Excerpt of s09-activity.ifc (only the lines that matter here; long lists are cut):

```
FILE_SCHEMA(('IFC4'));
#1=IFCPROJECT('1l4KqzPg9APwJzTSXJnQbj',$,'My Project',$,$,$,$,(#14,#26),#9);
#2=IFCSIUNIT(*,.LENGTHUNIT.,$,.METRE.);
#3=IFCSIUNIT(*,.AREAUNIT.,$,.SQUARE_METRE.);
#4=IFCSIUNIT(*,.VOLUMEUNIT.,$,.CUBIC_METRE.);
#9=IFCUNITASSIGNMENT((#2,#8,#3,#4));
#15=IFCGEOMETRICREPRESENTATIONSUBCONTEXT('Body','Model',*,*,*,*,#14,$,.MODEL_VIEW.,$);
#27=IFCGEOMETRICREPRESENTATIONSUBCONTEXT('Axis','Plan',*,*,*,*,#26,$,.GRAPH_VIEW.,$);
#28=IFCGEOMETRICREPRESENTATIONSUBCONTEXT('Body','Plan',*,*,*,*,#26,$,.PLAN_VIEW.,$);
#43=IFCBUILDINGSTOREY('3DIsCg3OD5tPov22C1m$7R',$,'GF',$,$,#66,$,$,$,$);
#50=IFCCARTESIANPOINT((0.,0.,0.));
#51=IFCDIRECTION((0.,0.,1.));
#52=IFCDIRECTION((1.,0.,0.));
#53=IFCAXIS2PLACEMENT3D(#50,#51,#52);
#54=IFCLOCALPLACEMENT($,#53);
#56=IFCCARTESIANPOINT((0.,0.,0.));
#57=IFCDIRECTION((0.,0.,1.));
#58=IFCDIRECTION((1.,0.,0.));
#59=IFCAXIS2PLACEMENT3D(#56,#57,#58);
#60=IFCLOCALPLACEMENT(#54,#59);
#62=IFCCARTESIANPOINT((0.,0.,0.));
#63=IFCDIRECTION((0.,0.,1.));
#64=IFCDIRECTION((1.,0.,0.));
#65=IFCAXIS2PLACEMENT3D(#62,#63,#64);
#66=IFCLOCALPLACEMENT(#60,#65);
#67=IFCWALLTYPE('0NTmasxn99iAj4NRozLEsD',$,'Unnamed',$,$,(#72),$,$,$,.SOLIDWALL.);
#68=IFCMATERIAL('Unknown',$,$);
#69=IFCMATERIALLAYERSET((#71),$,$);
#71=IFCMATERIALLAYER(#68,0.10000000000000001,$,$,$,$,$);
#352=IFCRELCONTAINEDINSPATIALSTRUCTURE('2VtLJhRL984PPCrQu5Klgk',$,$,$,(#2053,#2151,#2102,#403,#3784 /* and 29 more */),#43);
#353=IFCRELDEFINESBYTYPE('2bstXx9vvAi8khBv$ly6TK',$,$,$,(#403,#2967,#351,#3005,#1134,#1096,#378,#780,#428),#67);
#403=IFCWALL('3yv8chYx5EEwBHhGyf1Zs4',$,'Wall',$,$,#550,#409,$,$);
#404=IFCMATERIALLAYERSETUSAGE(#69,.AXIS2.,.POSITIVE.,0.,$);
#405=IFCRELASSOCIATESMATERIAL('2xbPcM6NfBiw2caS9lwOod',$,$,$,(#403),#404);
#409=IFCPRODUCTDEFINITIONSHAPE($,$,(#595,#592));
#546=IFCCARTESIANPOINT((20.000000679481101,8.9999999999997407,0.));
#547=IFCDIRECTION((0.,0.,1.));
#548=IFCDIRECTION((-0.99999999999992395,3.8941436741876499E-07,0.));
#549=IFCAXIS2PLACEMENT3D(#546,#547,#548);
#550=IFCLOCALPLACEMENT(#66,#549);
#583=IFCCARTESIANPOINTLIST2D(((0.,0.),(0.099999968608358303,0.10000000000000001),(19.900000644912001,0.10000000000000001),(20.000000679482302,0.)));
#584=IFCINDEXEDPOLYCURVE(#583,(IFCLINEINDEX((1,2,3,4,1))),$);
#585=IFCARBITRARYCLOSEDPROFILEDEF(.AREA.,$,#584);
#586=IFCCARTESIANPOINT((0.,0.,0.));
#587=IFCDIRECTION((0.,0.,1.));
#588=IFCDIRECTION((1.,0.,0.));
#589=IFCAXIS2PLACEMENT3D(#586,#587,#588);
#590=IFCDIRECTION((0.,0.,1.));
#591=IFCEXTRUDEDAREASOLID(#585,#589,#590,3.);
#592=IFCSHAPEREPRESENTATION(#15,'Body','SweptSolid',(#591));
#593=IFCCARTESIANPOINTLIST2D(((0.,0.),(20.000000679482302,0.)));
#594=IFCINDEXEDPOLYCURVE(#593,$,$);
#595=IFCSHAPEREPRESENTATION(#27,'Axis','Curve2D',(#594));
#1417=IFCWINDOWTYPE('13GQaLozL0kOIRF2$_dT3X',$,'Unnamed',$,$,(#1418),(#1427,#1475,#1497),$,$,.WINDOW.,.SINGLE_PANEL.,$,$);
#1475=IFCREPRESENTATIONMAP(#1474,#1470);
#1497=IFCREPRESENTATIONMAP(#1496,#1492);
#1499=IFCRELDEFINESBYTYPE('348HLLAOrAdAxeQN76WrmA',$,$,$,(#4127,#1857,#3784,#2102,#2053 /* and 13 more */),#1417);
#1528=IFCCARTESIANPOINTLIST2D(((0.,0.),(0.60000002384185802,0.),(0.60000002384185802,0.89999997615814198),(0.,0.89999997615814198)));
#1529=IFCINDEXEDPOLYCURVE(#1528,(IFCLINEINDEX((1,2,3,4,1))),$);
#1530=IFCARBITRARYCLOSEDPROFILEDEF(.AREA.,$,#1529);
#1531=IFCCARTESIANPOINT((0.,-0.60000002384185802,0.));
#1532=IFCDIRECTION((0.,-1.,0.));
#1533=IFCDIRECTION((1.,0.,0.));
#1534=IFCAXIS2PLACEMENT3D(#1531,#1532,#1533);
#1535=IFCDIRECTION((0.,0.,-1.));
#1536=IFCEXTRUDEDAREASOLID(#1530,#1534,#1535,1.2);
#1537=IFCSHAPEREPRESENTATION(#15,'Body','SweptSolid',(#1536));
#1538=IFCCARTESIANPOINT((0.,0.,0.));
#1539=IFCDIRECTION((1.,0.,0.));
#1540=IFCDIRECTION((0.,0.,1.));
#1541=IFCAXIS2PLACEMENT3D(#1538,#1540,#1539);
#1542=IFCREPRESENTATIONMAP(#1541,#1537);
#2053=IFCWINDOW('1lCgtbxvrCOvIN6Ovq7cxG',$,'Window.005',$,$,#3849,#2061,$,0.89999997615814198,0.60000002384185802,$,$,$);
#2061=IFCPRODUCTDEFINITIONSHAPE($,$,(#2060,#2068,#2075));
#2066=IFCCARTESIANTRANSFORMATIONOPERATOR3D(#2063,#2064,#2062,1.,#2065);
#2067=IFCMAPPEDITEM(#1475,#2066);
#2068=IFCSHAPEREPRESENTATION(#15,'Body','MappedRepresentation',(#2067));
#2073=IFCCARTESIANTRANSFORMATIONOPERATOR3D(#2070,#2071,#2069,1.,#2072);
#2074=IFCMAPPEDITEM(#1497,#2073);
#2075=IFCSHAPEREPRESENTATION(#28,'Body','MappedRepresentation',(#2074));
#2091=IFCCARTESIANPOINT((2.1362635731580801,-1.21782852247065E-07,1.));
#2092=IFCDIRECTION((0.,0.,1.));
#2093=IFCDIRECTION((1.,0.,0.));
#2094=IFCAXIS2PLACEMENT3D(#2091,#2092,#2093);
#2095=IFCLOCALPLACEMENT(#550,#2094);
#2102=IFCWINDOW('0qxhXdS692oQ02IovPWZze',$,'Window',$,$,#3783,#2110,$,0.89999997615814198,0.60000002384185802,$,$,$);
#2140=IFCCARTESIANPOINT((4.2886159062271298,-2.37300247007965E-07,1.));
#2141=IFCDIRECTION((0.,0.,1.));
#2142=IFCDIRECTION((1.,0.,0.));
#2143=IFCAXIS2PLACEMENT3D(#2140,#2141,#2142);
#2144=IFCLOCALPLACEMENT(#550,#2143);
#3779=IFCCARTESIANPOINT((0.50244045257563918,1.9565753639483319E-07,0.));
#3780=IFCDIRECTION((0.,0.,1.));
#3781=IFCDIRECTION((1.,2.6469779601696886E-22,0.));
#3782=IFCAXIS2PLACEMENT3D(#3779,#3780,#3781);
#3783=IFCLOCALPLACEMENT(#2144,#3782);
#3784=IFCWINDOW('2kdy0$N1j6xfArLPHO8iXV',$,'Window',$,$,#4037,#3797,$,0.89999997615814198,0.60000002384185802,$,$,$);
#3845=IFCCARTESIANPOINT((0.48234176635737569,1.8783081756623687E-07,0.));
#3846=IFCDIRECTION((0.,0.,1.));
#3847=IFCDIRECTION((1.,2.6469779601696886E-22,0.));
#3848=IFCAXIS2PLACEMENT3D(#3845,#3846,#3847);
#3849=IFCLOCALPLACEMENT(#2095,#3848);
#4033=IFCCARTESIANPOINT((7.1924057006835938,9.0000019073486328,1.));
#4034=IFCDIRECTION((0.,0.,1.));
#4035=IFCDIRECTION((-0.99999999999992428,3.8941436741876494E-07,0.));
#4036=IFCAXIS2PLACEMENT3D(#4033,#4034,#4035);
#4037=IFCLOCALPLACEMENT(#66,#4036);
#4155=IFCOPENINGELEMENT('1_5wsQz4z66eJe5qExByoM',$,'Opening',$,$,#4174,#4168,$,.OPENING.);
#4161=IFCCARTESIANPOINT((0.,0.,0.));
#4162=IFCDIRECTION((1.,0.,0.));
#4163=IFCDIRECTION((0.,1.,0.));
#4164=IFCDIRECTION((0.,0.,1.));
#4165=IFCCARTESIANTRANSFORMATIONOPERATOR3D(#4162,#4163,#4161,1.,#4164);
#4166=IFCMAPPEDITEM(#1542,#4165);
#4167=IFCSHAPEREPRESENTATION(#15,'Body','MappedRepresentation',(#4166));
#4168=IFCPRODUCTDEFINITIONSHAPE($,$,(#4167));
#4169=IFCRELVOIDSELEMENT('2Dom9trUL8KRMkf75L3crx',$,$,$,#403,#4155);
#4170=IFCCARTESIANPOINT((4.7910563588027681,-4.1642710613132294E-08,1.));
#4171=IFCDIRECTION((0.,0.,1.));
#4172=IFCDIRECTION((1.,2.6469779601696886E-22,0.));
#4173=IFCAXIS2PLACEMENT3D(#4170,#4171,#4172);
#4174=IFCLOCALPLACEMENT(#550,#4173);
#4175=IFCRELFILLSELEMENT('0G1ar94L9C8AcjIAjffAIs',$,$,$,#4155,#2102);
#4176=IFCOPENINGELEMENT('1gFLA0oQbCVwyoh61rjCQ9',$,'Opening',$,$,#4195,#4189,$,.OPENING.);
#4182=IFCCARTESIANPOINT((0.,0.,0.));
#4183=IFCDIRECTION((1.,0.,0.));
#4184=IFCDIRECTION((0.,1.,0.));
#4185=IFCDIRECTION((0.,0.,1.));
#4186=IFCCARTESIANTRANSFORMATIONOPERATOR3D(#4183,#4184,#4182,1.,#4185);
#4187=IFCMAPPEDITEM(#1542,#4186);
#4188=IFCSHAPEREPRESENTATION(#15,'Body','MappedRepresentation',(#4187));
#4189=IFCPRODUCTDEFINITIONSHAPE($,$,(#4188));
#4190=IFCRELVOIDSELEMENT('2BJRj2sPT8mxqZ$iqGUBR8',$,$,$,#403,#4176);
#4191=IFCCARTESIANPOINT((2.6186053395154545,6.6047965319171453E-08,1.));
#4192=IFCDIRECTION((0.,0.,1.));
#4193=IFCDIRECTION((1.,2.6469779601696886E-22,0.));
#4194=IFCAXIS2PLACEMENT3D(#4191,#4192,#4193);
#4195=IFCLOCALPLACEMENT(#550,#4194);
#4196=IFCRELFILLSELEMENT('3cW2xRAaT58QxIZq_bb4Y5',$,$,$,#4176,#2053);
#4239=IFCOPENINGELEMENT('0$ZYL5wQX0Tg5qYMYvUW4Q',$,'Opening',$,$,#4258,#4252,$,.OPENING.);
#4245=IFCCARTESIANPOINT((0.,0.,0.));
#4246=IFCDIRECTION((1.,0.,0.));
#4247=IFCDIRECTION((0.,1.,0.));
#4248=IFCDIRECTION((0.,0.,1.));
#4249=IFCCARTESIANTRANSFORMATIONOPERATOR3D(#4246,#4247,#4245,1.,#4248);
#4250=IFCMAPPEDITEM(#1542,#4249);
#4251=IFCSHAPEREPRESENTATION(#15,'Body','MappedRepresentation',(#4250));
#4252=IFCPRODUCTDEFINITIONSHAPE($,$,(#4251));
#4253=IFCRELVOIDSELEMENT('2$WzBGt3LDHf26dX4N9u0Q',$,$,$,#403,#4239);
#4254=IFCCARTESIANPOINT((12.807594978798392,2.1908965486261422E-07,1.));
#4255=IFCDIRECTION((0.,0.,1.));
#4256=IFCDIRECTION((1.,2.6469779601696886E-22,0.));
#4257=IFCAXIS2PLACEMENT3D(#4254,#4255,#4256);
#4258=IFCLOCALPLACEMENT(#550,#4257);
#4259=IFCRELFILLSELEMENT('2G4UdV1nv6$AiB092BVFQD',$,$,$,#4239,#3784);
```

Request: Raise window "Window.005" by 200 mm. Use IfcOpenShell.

```python
import numpy as np
import ifcopenshell
import ifcopenshell.api.geometry
import ifcopenshell.util.placement
import ifcopenshell.util.unit

model = ifcopenshell.open("s09-activity.ifc")
unit_scale = ifcopenshell.util.unit.calculate_unit_scale(model)

window = model.by_id(2053)
opening = window.FillsVoids[0].RelatingOpeningElement
dz = 0.2 / unit_scale

shift = np.array([0.0, 0.0, dz])
# The window is not placed relative to its opening, so move both.
for product in (opening, window):
    matrix = ifcopenshell.util.placement.get_local_placement(product.ObjectPlacement)
    matrix[:3, 3] += shift
    ifcopenshell.api.geometry.edit_object_placement(model, product=product, matrix=matrix, is_si=False)

print(f"moved by {dz * unit_scale:+.3f} m")

model.write("s09-activity_updated.ifc")
```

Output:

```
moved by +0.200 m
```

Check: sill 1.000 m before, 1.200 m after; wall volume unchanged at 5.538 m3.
